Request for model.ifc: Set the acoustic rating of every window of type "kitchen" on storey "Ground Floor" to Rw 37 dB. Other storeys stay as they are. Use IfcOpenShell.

First a look at what the model holds.

```python
import ifcopenshell
import ifcopenshell.util.element

model = ifcopenshell.open("model.ifc")
print(model.schema)
storey = next(s for s in model.by_type("IfcBuildingStorey") if s.Name == "Ground Floor")
windows = [e for e in ifcopenshell.util.element.get_decomposition(storey) if e.is_a("IfcWindow")]
seen = {}
for e in windows:
    element_type = ifcopenshell.util.element.get_type(e)
    key = (element_type.Name if element_type != e and element_type else None, ifcopenshell.util.element.get_pset(e, "Pset_WindowCommon", "AcousticRating"))
    seen[key] = seen.get(key, 0) + 1
for (name, value), count in sorted(seen.items(), key=str):
    print(count, "x", name, "|", value)
```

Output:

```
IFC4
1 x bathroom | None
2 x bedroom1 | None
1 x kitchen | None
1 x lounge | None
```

```python
import ifcopenshell
import ifcopenshell.api.pset
import ifcopenshell.util.element

model = ifcopenshell.open("model.ifc")

storey = next(s for s in model.by_type("IfcBuildingStorey") if s.Name == "Ground Floor")
windows = [e for e in ifcopenshell.util.element.get_decomposition(storey) if e.is_a("IfcWindow")]

count = 0
for e in windows:
    element_type = ifcopenshell.util.element.get_type(e)
    if element_type in (None, e) or element_type.Name != "kitchen":
        continue
    # add_pset returns the element's existing set when there is one.
    pset = ifcopenshell.api.pset.add_pset(model, product=e, name="Pset_WindowCommon")
    ifcopenshell.api.pset.edit_pset(model, pset=pset, properties={"AcousticRating": "Rw 37 dB"})
    count += 1

print(count, "windows updated")

model.write("model_rev.ifc")
```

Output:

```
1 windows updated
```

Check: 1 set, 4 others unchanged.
